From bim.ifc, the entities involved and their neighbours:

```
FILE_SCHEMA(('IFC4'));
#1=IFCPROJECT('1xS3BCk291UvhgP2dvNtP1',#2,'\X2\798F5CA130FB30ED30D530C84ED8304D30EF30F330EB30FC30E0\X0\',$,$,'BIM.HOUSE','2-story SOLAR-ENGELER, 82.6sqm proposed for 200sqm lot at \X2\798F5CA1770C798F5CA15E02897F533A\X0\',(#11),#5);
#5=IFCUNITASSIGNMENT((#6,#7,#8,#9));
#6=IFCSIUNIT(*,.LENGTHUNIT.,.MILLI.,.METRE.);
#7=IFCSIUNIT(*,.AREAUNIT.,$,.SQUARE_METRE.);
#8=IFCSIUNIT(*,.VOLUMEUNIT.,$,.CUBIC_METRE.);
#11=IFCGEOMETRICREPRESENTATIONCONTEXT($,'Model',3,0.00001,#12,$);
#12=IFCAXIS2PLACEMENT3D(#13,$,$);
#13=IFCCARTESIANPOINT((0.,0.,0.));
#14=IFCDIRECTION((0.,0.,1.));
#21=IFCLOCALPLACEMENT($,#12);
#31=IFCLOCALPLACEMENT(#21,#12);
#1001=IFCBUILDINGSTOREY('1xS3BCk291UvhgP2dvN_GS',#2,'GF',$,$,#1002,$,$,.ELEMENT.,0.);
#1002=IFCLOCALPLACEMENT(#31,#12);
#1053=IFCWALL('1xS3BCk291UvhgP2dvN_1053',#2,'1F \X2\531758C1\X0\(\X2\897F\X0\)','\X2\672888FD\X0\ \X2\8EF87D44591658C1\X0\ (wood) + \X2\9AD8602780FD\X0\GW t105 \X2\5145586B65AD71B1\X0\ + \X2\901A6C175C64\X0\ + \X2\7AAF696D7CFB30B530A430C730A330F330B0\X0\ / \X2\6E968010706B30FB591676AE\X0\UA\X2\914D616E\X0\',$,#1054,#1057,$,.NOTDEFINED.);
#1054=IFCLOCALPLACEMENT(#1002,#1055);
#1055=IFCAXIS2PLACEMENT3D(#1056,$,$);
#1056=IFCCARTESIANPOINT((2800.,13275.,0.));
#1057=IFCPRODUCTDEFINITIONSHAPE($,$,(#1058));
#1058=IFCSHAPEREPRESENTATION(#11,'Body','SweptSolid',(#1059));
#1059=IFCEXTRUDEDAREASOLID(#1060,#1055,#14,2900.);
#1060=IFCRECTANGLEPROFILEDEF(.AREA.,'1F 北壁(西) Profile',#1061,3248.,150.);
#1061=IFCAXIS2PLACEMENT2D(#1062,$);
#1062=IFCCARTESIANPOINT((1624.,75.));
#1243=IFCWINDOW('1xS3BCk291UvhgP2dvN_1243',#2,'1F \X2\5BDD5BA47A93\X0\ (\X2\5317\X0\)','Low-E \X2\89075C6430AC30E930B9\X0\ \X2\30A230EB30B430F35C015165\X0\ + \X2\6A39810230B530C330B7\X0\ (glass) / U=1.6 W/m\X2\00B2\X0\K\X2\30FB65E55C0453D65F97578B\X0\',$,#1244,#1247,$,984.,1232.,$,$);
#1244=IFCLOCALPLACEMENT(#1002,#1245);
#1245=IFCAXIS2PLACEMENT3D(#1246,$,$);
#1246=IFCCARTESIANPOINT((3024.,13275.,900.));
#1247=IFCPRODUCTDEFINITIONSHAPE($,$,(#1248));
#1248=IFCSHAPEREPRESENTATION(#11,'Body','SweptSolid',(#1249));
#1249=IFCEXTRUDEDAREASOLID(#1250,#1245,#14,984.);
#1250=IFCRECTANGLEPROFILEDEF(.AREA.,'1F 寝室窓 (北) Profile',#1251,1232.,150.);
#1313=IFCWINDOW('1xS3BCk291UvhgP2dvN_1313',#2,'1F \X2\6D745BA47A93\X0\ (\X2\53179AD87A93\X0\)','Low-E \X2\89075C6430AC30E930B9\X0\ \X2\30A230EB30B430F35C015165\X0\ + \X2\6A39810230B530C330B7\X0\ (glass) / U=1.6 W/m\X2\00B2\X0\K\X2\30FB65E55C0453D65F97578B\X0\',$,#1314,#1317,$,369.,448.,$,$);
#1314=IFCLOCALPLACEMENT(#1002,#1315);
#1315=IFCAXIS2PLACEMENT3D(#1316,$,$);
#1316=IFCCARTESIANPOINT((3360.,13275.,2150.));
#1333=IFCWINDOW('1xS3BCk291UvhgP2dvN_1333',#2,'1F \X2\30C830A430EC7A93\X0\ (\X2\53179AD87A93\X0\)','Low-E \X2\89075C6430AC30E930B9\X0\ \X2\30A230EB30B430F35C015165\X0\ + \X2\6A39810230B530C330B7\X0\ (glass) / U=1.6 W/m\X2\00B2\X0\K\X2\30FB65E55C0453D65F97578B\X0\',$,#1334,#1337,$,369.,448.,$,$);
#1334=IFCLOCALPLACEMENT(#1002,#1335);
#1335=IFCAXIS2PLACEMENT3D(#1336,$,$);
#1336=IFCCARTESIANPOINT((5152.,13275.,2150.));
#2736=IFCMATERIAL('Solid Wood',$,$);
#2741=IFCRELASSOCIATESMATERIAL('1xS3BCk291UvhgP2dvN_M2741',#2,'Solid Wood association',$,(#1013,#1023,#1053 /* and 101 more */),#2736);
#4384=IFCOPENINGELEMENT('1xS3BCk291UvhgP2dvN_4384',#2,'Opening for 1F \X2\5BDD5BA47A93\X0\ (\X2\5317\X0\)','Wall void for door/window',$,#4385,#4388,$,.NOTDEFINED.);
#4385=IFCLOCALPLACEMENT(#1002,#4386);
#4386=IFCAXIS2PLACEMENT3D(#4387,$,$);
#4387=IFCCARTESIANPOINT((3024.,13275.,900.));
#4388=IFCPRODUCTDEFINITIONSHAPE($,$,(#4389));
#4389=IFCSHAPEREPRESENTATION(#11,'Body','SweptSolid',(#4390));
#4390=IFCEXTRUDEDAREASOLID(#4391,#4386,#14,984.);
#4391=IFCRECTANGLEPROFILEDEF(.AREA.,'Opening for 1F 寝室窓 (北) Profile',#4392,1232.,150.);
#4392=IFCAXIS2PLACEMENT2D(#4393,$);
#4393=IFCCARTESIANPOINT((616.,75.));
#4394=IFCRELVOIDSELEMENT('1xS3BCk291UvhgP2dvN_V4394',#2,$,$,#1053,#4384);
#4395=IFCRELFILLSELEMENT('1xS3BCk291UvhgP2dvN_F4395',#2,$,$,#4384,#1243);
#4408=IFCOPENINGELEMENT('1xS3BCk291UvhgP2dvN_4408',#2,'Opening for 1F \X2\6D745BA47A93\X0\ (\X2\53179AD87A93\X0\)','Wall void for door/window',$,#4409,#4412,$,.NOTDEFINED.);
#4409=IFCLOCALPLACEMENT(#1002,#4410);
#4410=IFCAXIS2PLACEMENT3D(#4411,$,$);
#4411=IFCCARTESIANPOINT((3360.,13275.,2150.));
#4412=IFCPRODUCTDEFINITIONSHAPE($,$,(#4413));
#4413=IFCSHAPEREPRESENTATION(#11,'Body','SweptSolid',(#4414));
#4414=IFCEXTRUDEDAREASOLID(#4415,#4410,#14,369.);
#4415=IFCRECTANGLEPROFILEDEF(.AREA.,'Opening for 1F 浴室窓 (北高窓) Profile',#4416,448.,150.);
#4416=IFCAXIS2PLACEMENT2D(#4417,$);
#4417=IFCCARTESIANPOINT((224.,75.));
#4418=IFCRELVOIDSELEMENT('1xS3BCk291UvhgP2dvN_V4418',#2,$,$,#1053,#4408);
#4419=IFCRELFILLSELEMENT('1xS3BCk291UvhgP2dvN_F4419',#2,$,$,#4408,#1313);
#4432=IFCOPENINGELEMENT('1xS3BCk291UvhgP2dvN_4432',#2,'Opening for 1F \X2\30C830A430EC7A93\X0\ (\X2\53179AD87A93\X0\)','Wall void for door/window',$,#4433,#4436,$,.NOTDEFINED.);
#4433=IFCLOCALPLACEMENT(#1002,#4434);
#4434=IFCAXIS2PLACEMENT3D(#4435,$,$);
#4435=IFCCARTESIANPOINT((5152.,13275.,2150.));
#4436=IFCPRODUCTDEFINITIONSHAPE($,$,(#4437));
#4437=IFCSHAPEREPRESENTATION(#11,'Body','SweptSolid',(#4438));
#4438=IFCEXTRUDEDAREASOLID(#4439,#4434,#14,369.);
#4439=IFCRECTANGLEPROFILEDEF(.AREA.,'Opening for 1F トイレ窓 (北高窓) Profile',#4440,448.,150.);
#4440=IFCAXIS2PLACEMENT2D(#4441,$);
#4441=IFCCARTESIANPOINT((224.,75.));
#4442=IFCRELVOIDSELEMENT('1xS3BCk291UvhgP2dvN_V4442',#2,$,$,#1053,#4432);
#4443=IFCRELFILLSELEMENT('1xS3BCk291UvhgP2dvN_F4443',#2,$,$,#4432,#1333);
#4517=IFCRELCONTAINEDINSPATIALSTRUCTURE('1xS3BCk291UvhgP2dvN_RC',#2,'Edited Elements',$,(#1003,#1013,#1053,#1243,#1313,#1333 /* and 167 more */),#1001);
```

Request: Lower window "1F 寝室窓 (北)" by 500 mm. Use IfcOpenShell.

```python
import numpy as np
import ifcopenshell
import ifcopenshell.api.geometry
import ifcopenshell.util.placement
import ifcopenshell.util.unit

model = ifcopenshell.open("bim.ifc")
unit_scale = ifcopenshell.util.unit.calculate_unit_scale(model)

window = model.by_guid("1xS3BCk291UvhgP2dvN_1243")
opening = window.FillsVoids[0].RelatingOpeningElement
dz = -0.5 / unit_scale

shift = np.array([0.0, 0.0, dz])
# The window is not placed relative to its opening, so move both.
for product in (opening, window):
    matrix = ifcopenshell.util.placement.get_local_placement(product.ObjectPlacement)
    matrix[:3, 3] += shift
    ifcopenshell.api.geometry.edit_object_placement(model, product=product, matrix=matrix, is_si=False)

print(f"moved by {dz * unit_scale:+.3f} m")

model.write("bim-out.ifc")
```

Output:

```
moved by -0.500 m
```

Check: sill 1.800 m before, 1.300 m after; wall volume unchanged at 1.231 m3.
